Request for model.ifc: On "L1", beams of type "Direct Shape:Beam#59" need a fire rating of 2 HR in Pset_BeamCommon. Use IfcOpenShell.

First a look at what the model holds.

```python
import ifcopenshell
import ifcopenshell.util.element

model = ifcopenshell.open("model.ifc")
print(model.schema)
storey = next(s for s in model.by_type("IfcBuildingStorey") if s.Name == "L1")
beams = [e for e in ifcopenshell.util.element.get_decomposition(storey) if e.is_a("IfcBeam")]
seen = {}
for e in beams:
    element_type = ifcopenshell.util.element.get_type(e)
    key = (element_type.Name if element_type != e and element_type else None, ifcopenshell.util.element.get_pset(e, "Pset_BeamCommon", "FireRating"))
    seen[key] = seen.get(key, 0) + 1
for (name, value), count in sorted(seen.items(), key=str):
    print(count, "x", name, "|", value)
```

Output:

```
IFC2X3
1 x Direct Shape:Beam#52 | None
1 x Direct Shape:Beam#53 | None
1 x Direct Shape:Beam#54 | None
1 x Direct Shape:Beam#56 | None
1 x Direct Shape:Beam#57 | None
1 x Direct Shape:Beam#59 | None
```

```python
import ifcopenshell
import ifcopenshell.api.pset
import ifcopenshell.util.element

model = ifcopenshell.open("model.ifc")

storey = next(s for s in model.by_type("IfcBuildingStorey") if s.Name == "L1")
beams = [e for e in ifcopenshell.util.element.get_decomposition(storey) if e.is_a("IfcBeam")]

count = 0
for e in beams:
    element_type = ifcopenshell.util.element.get_type(e)
    if element_type in (None, e) or element_type.Name != "Direct Shape:Beam#59":
        continue
    # add_pset returns the element's existing set when there is one.
    pset = ifcopenshell.api.pset.add_pset(model, product=e, name="Pset_BeamCommon")
    ifcopenshell.api.pset.edit_pset(model, pset=pset, properties={"FireRating": "2 HR"})
    count += 1

print(count, "beams updated")

model.write("model_v2.ifc")
```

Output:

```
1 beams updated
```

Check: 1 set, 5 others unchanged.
